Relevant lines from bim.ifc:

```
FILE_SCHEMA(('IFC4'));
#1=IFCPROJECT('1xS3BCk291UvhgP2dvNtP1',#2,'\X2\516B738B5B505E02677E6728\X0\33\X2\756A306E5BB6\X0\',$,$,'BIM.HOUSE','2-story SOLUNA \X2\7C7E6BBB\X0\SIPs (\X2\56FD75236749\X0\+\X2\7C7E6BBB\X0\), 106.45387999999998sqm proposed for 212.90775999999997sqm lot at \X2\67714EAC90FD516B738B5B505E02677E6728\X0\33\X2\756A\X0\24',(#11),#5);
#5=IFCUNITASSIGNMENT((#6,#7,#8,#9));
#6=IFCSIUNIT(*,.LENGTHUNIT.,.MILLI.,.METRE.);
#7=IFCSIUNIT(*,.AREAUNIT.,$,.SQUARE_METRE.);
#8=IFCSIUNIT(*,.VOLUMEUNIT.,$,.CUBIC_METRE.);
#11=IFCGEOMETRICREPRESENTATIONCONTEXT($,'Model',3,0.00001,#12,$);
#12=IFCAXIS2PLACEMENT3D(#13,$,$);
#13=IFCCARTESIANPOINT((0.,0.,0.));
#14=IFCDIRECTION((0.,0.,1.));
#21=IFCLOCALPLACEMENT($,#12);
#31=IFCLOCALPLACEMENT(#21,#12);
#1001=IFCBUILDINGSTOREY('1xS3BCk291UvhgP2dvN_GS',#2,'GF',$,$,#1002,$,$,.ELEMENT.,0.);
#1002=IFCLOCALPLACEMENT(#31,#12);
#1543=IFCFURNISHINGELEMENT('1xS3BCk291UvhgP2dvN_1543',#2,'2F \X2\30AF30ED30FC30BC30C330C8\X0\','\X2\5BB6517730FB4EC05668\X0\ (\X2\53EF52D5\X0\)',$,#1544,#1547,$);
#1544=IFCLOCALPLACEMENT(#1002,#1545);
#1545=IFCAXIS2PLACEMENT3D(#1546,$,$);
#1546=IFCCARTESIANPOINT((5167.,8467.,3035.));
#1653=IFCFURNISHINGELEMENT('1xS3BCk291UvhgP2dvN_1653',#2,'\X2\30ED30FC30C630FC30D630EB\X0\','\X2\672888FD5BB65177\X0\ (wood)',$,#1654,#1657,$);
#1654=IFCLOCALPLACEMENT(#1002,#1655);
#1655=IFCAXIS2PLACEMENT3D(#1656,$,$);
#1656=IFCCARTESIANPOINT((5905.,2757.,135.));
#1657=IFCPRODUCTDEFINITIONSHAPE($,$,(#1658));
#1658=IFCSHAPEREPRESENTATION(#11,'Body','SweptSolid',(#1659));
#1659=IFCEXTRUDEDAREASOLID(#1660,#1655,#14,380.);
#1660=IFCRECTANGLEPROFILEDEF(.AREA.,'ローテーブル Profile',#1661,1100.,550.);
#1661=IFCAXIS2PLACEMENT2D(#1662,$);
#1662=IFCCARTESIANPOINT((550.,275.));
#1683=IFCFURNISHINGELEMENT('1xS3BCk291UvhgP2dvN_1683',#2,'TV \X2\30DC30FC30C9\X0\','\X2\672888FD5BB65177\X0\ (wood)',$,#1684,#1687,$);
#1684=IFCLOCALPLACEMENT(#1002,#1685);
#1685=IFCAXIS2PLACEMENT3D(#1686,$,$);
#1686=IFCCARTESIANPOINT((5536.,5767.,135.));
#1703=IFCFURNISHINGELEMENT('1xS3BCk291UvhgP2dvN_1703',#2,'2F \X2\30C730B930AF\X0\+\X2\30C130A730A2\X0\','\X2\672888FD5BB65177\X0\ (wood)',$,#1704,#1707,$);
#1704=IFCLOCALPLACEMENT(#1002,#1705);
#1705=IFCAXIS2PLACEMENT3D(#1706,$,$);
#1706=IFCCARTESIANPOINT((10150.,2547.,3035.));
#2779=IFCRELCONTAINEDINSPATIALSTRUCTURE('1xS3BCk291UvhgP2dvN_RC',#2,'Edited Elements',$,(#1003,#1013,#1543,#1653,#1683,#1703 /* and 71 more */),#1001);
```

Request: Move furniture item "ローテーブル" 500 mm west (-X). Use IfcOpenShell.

```python
import ifcopenshell
import ifcopenshell.api.geometry
import ifcopenshell.util.placement

model = ifcopenshell.open("bim.ifc")

item = model.by_guid("1xS3BCk291UvhgP2dvN_1653")
matrix = ifcopenshell.util.placement.get_local_placement(item.ObjectPlacement)
matrix[0, 3] -= 500.0
ifcopenshell.api.geometry.edit_object_placement(model, product=item, matrix=matrix, is_si=False)

print(ifcopenshell.util.placement.get_local_placement(item.ObjectPlacement).round(3) + 0.0)

model.write("bim_rev.ifc")
```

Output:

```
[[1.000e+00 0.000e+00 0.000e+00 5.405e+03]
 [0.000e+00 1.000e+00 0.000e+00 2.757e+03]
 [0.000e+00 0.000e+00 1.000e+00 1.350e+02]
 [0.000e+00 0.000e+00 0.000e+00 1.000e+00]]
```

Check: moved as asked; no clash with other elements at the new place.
